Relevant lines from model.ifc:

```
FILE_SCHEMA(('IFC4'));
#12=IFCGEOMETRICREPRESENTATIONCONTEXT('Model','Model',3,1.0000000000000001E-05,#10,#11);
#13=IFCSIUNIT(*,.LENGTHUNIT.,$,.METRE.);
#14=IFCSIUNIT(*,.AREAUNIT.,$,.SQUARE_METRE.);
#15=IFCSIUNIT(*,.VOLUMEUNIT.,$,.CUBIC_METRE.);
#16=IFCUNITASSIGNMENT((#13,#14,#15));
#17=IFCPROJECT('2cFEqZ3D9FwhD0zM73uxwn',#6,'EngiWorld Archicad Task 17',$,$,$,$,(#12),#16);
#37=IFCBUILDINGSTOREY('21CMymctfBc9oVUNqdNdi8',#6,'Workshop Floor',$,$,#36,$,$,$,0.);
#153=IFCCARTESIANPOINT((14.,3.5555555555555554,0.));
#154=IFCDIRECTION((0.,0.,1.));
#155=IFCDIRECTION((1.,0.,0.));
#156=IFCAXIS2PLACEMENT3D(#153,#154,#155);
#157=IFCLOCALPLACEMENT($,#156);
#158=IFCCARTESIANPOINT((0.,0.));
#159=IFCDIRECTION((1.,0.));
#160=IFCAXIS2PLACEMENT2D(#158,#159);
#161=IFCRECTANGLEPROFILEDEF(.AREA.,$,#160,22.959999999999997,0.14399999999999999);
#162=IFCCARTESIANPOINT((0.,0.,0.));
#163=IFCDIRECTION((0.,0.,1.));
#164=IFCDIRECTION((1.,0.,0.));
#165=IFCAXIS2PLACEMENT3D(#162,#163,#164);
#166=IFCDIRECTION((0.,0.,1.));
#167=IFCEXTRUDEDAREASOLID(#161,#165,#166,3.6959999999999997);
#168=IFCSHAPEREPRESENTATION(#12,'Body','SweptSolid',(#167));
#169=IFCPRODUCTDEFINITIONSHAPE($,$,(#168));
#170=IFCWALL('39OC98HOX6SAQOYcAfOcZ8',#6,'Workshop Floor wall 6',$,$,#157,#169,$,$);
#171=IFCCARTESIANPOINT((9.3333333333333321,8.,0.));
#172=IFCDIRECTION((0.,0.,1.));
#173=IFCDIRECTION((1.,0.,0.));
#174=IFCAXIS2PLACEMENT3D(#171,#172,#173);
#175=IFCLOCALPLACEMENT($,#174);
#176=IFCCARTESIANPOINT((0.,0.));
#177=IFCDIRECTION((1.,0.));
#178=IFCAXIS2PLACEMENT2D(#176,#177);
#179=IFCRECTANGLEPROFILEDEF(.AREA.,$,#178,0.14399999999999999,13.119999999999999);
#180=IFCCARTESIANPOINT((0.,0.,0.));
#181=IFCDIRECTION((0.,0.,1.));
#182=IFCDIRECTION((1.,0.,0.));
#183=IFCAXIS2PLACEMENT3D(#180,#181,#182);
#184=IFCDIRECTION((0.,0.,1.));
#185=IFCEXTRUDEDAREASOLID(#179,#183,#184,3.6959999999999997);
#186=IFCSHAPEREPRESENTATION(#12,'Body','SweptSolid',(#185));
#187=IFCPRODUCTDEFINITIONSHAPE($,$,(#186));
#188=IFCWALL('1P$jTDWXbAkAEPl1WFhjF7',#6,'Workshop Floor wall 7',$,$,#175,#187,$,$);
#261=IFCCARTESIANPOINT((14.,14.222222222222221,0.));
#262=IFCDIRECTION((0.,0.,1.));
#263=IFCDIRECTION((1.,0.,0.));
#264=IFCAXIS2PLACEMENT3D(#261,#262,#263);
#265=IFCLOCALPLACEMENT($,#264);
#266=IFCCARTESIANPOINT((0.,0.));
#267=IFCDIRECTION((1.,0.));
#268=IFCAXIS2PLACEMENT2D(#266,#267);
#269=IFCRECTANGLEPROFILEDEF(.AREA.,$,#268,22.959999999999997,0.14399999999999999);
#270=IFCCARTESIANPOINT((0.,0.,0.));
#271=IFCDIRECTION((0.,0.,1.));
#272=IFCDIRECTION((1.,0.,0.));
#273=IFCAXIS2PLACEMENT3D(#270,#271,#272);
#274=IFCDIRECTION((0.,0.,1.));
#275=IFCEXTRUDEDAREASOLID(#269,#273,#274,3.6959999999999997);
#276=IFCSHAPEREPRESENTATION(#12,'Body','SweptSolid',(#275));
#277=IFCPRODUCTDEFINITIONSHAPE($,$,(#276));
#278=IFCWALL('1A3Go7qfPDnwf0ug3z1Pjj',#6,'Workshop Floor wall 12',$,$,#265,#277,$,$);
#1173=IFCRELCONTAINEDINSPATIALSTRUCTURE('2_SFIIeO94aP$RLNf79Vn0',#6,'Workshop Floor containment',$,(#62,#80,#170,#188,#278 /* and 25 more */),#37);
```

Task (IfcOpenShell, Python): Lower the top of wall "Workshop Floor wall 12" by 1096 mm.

```python
import ifcopenshell
import ifcopenshell.geom
import ifcopenshell.util.shape

model = ifcopenshell.open("model.ifc")
settings = ifcopenshell.geom.settings()


def volume(element):
    """Net volume in cubic metres, openings subtracted."""
    shape = ifcopenshell.geom.create_shape(settings, element)
    return ifcopenshell.util.shape.get_volume(shape.geometry)


wall = model.by_guid("1A3Go7qfPDnwf0ug3z1Pjj")
before = volume(wall)

body = next(r for r in wall.Representation.Representations if r.RepresentationIdentifier == "Body")
solid = body.Items[0]
old_height = solid.Depth
solid.Depth -= 1.096
after = volume(wall)

print(f"height {old_height:g} -> {solid.Depth:g}, volume {before:.3f} -> {after:.3f} m3")

model.write("model-out.ifc")
```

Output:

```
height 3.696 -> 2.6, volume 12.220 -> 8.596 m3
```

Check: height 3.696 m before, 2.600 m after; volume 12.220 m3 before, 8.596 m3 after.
